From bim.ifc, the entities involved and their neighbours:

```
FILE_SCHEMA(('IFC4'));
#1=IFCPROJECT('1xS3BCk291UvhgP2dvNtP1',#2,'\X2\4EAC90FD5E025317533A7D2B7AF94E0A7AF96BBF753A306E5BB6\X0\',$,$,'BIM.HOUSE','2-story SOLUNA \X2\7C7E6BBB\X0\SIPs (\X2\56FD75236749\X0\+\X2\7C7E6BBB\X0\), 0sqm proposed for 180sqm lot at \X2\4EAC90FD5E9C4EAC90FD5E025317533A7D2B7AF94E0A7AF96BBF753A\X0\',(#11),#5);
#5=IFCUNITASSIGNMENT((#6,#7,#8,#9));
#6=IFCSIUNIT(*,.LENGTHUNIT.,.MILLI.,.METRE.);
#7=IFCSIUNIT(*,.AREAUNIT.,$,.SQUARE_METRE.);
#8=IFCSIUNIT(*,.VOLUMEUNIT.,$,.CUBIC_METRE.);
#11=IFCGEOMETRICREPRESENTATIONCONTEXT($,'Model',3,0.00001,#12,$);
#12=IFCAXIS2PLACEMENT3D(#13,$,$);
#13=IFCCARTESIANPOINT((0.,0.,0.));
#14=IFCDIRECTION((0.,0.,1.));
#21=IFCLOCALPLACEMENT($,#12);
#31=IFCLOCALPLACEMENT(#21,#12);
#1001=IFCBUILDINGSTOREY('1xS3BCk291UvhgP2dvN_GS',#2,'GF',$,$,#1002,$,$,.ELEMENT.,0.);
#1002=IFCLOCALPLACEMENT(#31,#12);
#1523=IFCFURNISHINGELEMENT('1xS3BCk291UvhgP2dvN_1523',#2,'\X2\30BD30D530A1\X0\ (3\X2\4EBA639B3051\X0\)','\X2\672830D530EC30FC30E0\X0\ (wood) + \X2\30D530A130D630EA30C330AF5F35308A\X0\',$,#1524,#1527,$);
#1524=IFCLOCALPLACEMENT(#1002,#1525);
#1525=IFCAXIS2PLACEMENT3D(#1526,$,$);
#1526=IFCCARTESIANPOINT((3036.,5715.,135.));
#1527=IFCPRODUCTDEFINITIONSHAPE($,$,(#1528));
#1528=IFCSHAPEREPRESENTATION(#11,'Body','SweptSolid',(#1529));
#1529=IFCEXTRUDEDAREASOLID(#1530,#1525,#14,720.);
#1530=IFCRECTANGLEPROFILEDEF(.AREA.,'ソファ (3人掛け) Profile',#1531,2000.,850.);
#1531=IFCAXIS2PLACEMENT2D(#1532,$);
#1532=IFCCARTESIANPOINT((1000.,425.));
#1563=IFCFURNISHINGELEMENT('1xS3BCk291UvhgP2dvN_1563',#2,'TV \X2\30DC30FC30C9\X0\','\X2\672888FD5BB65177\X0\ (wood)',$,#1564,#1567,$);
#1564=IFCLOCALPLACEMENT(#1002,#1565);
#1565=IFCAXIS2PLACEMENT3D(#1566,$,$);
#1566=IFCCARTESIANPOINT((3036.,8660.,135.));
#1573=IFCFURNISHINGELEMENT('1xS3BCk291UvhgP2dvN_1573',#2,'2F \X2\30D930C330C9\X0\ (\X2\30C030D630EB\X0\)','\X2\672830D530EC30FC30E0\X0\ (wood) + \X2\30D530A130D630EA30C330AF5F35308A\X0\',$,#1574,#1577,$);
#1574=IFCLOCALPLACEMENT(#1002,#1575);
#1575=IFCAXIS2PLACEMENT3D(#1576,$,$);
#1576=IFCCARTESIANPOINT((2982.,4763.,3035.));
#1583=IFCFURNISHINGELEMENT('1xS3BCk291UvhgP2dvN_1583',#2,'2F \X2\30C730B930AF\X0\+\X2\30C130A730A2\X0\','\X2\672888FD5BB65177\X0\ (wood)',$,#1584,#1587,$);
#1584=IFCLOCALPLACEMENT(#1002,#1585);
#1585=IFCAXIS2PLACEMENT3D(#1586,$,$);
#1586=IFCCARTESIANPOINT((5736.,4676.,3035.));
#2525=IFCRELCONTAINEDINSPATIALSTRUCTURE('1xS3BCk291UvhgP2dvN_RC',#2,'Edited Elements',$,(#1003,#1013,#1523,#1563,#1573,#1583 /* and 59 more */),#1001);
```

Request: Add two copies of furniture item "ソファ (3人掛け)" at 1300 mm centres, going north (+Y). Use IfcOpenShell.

```python
import numpy as np
import ifcopenshell
import ifcopenshell.api.geometry
import ifcopenshell.api.root
import ifcopenshell.util.element
import ifcopenshell.util.placement

model = ifcopenshell.open("bim.ifc")


def reuse_history(source, copy):
    """copy_class also copies each property set's owner history, people and application; keep the originals."""
    for rel in copy.IsDefinedBy:
        if rel.is_a("IfcRelDefinesByProperties") and (history := rel.RelatingPropertyDefinition.OwnerHistory):
            rel.RelatingPropertyDefinition.OwnerHistory = source.OwnerHistory
            ifcopenshell.util.element.remove_deep2(model, history)


source = model.by_id(1523)
base = ifcopenshell.util.placement.get_local_placement(source.ObjectPlacement)
step = np.array([0.0, 1.0, 0.0]) * 1300.0

for i in range(1, 3):
    copy = ifcopenshell.api.root.copy_class(model, product=source)
    copy.Representation = ifcopenshell.util.element.copy_deep(
        model, source.Representation, exclude=["IfcGeometricRepresentationContext", "IfcRepresentationMap"]
    )
    reuse_history(source, copy)
    matrix = base.copy()
    matrix[:3, 3] += i * step
    print("added at", matrix[:3, 3].round(3) + 0.0)
    ifcopenshell.api.geometry.edit_object_placement(model, product=copy, matrix=matrix, is_si=False)

model.write("bim_updated.ifc")
```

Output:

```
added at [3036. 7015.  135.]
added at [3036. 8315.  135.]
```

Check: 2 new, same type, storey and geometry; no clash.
